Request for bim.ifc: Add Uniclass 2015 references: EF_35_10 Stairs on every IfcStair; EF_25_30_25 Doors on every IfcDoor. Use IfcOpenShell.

First a look at what the model holds.

```python
import ifcopenshell

model = ifcopenshell.open("bim.ifc")
print(model.schema)
print("classifications:", [c.Name for c in model.by_type("IfcClassification")])
for ifc_class in ("IfcDoor", "IfcRoof", "IfcStair", "IfcWall", "IfcWindow"):
    print(ifc_class, len(model.by_type(ifc_class)))
```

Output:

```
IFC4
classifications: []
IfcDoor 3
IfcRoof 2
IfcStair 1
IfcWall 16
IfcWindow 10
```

```python
import ifcopenshell
import ifcopenshell.api.classification

model = ifcopenshell.open("bim.ifc")

system = ifcopenshell.api.classification.add_classification(model, classification="Uniclass 2015")

codes = {
    "IfcStair": ("EF_35_10", "Stairs"),
    "IfcDoor": ("EF_25_30_25", "Doors"),
}
for ifc_class, (code, name) in codes.items():
    products = model.by_type(ifc_class)
    ifcopenshell.api.classification.add_reference(
        model, products=products, classification=system, identification=code, name=name
    )
    print(code, len(products))

model.write("bim_updated.ifc")
```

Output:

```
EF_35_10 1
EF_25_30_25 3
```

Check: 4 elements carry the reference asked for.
